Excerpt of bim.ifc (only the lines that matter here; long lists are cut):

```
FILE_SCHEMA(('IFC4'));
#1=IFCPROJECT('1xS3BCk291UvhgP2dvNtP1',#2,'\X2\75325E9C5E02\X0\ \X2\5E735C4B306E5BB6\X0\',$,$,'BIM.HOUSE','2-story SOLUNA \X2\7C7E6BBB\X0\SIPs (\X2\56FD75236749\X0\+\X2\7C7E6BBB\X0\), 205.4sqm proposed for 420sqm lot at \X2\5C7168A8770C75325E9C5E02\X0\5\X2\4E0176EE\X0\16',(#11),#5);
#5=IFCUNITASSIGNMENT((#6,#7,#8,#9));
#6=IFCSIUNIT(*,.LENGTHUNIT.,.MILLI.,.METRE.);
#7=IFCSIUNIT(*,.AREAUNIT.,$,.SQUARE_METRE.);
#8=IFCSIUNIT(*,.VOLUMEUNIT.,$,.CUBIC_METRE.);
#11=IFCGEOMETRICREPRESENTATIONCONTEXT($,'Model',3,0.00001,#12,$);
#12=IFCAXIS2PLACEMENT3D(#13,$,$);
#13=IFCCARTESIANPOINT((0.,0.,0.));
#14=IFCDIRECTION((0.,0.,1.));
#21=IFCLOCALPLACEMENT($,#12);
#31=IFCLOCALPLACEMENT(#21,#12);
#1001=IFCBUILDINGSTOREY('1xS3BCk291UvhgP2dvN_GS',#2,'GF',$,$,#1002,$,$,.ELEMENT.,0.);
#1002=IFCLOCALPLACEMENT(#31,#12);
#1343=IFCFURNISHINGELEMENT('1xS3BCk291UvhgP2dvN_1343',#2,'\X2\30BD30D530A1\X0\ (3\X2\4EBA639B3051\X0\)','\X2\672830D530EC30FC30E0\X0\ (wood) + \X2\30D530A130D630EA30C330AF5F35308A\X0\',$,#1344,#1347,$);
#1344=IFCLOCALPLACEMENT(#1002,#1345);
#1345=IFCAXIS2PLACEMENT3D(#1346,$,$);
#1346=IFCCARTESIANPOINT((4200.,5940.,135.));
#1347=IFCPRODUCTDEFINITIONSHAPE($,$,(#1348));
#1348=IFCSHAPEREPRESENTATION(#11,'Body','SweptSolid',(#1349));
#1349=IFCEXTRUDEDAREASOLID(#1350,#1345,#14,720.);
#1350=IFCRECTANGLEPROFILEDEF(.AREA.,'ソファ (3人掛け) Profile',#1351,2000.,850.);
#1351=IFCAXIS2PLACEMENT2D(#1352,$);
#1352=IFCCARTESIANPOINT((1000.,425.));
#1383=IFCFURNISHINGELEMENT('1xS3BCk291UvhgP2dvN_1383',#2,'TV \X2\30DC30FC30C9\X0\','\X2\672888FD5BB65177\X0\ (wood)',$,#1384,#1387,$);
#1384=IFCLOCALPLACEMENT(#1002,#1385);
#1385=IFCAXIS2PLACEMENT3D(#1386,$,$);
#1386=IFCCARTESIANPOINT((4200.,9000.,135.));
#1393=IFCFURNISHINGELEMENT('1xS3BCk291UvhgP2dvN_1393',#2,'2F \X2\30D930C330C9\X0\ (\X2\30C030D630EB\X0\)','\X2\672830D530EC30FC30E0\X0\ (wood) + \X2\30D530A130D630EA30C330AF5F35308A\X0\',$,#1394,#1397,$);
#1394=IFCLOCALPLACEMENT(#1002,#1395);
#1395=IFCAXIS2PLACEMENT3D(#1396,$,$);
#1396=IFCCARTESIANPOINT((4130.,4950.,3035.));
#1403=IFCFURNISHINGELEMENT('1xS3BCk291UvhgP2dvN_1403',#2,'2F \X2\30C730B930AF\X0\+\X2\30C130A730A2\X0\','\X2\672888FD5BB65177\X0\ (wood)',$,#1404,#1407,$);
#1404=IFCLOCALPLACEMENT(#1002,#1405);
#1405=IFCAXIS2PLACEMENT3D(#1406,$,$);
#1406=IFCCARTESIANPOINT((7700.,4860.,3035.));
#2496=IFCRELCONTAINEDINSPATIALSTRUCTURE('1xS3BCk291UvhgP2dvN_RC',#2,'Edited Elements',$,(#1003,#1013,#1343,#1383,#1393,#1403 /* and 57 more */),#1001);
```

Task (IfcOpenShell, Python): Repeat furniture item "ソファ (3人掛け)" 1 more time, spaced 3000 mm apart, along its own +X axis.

```python
import ifcopenshell
import ifcopenshell.api.geometry
import ifcopenshell.api.root
import ifcopenshell.util.element
import ifcopenshell.util.placement

model = ifcopenshell.open("bim.ifc")


def reuse_history(source, copy):
    """copy_class also copies each property set's owner history, people and application; keep the originals."""
    for rel in copy.IsDefinedBy:
        if rel.is_a("IfcRelDefinesByProperties") and (history := rel.RelatingPropertyDefinition.OwnerHistory):
            rel.RelatingPropertyDefinition.OwnerHistory = source.OwnerHistory
            ifcopenshell.util.element.remove_deep2(model, history)


source = model.by_guid("1xS3BCk291UvhgP2dvN_1343")
base = ifcopenshell.util.placement.get_local_placement(source.ObjectPlacement)
step = base[:3, 0] * 3000.0

for i in range(1, 2):
    copy = ifcopenshell.api.root.copy_class(model, product=source)
    copy.Representation = ifcopenshell.util.element.copy_deep(
        model, source.Representation, exclude=["IfcGeometricRepresentationContext", "IfcRepresentationMap"]
    )
    reuse_history(source, copy)
    matrix = base.copy()
    matrix[:3, 3] += i * step
    print("added at", matrix[:3, 3].round(3) + 0.0)
    ifcopenshell.api.geometry.edit_object_placement(model, product=copy, matrix=matrix, is_si=False)

model.write("bim_updated.ifc")
```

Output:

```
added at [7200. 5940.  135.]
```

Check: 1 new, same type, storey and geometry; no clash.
